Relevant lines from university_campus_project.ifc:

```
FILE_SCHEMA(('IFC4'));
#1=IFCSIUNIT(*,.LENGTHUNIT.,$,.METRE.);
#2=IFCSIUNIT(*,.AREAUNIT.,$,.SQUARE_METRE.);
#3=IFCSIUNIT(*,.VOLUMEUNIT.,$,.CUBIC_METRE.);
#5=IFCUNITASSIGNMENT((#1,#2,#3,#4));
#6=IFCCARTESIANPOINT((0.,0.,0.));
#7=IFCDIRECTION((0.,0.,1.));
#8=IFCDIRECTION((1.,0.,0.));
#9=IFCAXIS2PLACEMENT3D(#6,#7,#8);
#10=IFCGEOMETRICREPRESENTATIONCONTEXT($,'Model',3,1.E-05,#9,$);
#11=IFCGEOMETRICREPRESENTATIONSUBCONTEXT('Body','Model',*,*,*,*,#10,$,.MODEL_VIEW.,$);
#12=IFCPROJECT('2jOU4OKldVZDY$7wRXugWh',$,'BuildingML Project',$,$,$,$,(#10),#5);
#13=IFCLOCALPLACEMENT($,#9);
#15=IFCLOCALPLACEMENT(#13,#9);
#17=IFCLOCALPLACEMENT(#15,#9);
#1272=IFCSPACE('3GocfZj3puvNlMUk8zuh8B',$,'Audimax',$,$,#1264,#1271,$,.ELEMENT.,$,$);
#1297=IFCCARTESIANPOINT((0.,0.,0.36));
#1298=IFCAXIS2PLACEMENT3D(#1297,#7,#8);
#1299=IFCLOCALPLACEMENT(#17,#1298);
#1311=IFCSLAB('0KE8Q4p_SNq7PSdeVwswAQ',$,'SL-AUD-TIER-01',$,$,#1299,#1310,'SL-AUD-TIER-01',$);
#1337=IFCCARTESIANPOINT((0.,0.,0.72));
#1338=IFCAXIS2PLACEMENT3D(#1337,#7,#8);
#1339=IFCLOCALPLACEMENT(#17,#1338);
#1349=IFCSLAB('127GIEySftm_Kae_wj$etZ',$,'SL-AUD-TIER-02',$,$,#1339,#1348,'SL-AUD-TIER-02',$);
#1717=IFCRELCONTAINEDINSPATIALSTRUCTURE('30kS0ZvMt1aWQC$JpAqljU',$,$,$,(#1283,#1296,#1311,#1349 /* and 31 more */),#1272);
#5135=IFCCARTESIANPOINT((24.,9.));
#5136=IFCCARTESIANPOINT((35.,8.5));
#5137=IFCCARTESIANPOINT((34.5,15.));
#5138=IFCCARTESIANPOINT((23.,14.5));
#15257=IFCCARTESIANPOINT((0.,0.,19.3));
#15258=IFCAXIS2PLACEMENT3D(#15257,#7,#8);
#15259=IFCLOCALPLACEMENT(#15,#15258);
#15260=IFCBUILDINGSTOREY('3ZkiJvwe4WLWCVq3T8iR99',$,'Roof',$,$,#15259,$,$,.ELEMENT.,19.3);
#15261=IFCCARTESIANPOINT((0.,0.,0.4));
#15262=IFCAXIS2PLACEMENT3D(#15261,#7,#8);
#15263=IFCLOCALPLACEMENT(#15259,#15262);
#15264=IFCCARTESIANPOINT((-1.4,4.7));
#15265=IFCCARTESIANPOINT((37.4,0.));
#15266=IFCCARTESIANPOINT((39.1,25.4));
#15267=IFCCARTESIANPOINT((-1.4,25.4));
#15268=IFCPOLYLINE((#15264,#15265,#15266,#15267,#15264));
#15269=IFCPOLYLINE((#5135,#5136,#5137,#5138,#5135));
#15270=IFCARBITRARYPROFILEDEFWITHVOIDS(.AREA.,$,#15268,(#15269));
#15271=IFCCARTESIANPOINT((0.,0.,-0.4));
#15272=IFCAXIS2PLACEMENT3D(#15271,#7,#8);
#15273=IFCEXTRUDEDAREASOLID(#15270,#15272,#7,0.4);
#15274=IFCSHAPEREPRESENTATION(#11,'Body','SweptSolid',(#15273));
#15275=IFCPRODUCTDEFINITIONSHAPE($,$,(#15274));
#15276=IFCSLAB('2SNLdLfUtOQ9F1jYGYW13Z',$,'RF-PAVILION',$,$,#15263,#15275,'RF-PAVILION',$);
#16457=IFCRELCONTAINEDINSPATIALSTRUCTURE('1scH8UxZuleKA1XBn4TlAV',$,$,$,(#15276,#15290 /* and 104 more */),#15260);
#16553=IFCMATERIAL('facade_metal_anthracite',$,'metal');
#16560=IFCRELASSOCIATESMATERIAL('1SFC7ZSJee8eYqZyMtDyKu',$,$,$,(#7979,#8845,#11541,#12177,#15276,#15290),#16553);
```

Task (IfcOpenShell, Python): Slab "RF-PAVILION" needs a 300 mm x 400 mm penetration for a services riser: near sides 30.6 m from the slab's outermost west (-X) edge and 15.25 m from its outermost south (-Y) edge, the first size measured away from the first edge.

```python
import numpy as np
import ifcopenshell
import ifcopenshell.api.feature
import ifcopenshell.api.geometry
import ifcopenshell.api.root
import ifcopenshell.geom
import ifcopenshell.util.placement
import ifcopenshell.util.representation
import ifcopenshell.util.shape
import ifcopenshell.util.unit

model = ifcopenshell.open("university_campus_project.ifc")
unit_scale = ifcopenshell.util.unit.calculate_unit_scale(model)
settings = ifcopenshell.geom.settings()


def volume(element):
    """Net volume in cubic metres, openings subtracted."""
    shape = ifcopenshell.geom.create_shape(settings, element)
    return ifcopenshell.util.shape.get_volume(shape.geometry)


slab = model.by_guid("2SNLdLfUtOQ9F1jYGYW13Z")
before = volume(slab)

# Extent in the slab's own axes, in metres. The edges named are its -X and -Y sides.
slab_shape = ifcopenshell.geom.create_shape(settings, slab)
vertices = ifcopenshell.util.shape.get_vertices(slab_shape.geometry)
x_min, y_min, bottom = vertices.min(axis=0)
top = vertices[:, 2].max()

opening = ifcopenshell.api.root.create_entity(model, ifc_class="IfcOpeningElement", name="Services riser opening", predefined_type="OPENING")
context = ifcopenshell.util.representation.get_context(model, "Model", "Body", "MODEL_VIEW")
width, depth = 0.3, 0.4
outline = [(0.0, 0.0), (width, 0.0), (width, depth), (0.0, depth), (0.0, 0.0)]
# Overshoot both faces by 50 mm so the cut is clean.
shape = ifcopenshell.api.geometry.add_slab_representation(
    model, context=context, depth=top - bottom + 0.1, polyline=outline
)
ifcopenshell.api.geometry.assign_representation(model, product=opening, representation=shape)

matrix = ifcopenshell.util.placement.get_local_placement(slab.ObjectPlacement)
matrix[:, 3] = matrix @ np.append(np.array([x_min + 30.6, y_min + 15.25, bottom - 0.05]) / unit_scale, 1.0)
ifcopenshell.api.geometry.edit_object_placement(model, product=opening, matrix=matrix, is_si=False)
ifcopenshell.api.feature.add_feature(model, feature=opening, element=slab)

after = volume(slab)

print(f"slab volume {before:.3f} -> {after:.3f} m3")

model.write("university_campus_project_edited.ifc")
```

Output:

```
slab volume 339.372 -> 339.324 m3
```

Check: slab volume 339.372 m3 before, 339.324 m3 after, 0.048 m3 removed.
